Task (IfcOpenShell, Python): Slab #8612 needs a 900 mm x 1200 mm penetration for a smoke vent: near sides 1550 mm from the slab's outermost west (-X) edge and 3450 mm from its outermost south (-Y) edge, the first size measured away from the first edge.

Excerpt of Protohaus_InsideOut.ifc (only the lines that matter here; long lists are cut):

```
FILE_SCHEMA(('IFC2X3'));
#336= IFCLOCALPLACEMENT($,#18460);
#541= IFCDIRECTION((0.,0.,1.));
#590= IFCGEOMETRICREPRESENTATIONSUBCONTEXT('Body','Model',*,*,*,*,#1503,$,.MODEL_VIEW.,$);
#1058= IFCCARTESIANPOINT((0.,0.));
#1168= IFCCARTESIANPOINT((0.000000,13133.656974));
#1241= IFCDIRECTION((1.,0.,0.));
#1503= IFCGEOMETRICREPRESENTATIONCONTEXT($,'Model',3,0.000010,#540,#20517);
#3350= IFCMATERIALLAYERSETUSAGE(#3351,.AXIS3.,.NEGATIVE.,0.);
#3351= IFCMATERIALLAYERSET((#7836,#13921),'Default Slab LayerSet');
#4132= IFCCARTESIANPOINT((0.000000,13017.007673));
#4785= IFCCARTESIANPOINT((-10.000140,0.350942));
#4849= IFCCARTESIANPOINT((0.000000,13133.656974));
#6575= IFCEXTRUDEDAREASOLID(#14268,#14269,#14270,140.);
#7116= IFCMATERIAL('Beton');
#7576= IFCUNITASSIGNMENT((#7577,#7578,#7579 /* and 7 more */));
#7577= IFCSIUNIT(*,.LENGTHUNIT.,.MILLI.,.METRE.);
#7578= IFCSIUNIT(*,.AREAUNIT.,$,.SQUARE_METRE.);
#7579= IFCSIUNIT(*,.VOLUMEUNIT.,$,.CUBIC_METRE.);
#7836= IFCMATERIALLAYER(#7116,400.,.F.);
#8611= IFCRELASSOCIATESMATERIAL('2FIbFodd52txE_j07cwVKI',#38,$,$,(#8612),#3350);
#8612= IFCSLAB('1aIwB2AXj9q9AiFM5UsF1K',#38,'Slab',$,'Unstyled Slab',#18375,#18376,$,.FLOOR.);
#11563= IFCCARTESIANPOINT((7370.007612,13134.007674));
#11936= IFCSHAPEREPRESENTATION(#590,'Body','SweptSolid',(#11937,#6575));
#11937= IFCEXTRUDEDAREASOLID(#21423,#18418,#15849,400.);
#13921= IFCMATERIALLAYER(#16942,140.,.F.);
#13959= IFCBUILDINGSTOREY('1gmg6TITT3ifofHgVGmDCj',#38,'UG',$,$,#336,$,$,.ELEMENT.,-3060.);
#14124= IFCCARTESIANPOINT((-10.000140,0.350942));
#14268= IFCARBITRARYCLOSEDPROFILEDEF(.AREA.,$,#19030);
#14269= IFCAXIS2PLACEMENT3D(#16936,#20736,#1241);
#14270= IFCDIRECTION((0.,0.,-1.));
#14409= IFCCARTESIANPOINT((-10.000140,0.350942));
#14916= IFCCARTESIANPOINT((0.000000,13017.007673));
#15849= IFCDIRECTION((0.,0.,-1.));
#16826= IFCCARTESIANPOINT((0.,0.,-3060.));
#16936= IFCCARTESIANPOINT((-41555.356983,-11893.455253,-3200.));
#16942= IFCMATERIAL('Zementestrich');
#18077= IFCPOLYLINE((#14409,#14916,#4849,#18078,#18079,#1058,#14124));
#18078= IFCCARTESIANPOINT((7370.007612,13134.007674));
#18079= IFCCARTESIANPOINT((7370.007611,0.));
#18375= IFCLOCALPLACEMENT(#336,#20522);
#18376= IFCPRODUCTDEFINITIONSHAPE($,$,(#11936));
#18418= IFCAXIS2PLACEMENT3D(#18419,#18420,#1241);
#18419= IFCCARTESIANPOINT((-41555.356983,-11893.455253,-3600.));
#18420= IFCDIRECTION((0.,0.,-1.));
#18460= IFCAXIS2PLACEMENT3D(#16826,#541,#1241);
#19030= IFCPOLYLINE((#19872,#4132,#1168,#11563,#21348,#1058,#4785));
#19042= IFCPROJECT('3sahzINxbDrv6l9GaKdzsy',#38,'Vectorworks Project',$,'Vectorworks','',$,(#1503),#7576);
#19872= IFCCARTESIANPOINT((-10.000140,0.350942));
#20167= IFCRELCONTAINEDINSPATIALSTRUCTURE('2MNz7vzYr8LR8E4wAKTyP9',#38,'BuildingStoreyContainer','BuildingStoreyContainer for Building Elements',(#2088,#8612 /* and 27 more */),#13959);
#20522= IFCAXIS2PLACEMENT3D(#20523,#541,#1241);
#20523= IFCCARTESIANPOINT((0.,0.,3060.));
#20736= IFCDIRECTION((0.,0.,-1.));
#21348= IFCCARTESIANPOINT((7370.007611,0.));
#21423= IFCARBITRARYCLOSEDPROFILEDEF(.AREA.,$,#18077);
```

```python
import numpy as np
import ifcopenshell
import ifcopenshell.api.feature
import ifcopenshell.api.geometry
import ifcopenshell.api.root
import ifcopenshell.geom
import ifcopenshell.util.placement
import ifcopenshell.util.representation
import ifcopenshell.util.shape
import ifcopenshell.util.unit

model = ifcopenshell.open("Protohaus_InsideOut.ifc")
unit_scale = ifcopenshell.util.unit.calculate_unit_scale(model)
settings = ifcopenshell.geom.settings()


def volume(element):
    """Net volume in cubic metres, openings subtracted."""
    shape = ifcopenshell.geom.create_shape(settings, element)
    return ifcopenshell.util.shape.get_volume(shape.geometry)


slab = model.by_guid("1aIwB2AXj9q9AiFM5UsF1K")
before = volume(slab)

# Extent in the slab's own axes, in metres. The edges named are its -X and -Y sides.
slab_shape = ifcopenshell.geom.create_shape(settings, slab)
vertices = ifcopenshell.util.shape.get_vertices(slab_shape.geometry)
x_min, y_min, bottom = vertices.min(axis=0)
top = vertices[:, 2].max()

opening = ifcopenshell.api.root.create_entity(model, ifc_class="IfcOpeningElement", name="Smoke vent opening")
context = ifcopenshell.util.representation.get_context(model, "Model", "Body", "MODEL_VIEW")
width, depth = 0.9, 1.2
outline = [(0.0, 0.0), (width, 0.0), (width, depth), (0.0, depth), (0.0, 0.0)]
# Overshoot both faces by 50 mm so the cut is clean.
shape = ifcopenshell.api.geometry.add_slab_representation(
    model, context=context, depth=top - bottom + 0.1, polyline=outline
)
ifcopenshell.api.geometry.assign_representation(model, product=opening, representation=shape)

matrix = ifcopenshell.util.placement.get_local_placement(slab.ObjectPlacement)
matrix[:, 3] = matrix @ np.append(np.array([x_min + 1.55, y_min + 3.45, bottom - 0.05]) / unit_scale, 1.0)
ifcopenshell.api.geometry.edit_object_placement(model, product=opening, matrix=matrix, is_si=False)
ifcopenshell.api.feature.add_feature(model, feature=opening, element=slab)

after = volume(slab)

print(f"slab volume {before:.3f} -> {after:.3f} m3")

model.write("Protohaus_InsideOut_v2.ifc")
```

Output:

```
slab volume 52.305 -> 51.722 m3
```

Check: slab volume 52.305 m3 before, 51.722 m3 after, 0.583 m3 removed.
